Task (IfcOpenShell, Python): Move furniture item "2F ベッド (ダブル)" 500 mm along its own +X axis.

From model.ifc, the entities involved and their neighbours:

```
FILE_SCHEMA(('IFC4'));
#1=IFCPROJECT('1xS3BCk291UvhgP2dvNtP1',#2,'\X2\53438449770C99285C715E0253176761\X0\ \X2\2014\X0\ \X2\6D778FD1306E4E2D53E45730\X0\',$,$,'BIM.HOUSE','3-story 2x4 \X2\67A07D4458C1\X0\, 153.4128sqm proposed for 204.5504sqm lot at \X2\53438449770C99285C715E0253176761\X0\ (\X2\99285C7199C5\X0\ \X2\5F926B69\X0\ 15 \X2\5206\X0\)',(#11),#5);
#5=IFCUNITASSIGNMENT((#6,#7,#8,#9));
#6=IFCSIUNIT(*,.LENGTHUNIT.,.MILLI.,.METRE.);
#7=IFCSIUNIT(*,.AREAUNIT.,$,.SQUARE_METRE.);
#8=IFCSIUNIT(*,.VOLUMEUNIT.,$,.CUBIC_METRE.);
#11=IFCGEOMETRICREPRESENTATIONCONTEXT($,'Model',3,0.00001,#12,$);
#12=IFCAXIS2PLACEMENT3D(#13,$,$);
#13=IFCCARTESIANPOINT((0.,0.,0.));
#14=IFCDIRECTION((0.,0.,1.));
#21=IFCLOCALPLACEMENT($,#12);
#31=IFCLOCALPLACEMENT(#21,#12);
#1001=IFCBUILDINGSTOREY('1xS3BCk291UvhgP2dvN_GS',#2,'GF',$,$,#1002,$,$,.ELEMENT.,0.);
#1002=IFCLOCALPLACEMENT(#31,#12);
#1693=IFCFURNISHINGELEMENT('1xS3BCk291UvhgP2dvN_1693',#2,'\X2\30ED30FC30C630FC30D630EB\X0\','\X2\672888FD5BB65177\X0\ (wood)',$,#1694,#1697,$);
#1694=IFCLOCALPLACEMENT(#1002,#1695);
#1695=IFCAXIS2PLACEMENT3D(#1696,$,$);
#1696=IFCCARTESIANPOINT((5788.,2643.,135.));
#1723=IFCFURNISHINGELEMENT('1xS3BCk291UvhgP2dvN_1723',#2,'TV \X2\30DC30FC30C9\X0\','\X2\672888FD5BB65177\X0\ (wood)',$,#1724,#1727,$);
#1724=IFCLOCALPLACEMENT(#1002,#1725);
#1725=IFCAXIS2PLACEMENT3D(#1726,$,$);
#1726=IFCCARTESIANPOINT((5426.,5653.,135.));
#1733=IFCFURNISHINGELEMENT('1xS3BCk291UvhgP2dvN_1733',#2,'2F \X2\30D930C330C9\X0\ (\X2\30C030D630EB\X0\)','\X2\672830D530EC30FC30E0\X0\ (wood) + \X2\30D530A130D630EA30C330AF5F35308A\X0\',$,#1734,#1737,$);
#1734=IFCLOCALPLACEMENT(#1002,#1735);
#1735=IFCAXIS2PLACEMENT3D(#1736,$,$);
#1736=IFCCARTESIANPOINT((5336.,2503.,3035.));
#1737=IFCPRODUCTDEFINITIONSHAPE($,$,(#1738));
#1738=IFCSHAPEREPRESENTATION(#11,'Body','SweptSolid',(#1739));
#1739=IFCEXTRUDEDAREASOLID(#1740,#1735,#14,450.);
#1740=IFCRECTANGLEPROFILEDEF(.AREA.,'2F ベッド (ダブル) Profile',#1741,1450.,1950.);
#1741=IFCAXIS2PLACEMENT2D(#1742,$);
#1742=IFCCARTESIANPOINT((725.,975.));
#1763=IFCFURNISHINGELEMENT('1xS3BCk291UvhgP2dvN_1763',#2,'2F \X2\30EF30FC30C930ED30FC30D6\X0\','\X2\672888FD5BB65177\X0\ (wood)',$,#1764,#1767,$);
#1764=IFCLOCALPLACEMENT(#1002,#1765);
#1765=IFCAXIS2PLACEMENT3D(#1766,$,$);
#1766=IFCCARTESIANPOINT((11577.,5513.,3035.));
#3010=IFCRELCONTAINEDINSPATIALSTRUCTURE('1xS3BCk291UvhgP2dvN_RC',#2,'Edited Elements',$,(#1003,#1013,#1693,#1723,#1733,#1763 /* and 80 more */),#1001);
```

```python
import ifcopenshell
import ifcopenshell.api.geometry
import ifcopenshell.util.placement
import ifcopenshell.util.unit

model = ifcopenshell.open("model.ifc")
unit_scale = ifcopenshell.util.unit.calculate_unit_scale(model)

item = model.by_guid("1xS3BCk291UvhgP2dvN_1733")
matrix = ifcopenshell.util.placement.get_local_placement(item.ObjectPlacement)
matrix[:3, 3] += matrix[:3, 0] * 0.5 / unit_scale
ifcopenshell.api.geometry.edit_object_placement(model, product=item, matrix=matrix, is_si=False)

print(ifcopenshell.util.placement.get_local_placement(item.ObjectPlacement).round(3) + 0.0)

model.write("model_edited.ifc")
```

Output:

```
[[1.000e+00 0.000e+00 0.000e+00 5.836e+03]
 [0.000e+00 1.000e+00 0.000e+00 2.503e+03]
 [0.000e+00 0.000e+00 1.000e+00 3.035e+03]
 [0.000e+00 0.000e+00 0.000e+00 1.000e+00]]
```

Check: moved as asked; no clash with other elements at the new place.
